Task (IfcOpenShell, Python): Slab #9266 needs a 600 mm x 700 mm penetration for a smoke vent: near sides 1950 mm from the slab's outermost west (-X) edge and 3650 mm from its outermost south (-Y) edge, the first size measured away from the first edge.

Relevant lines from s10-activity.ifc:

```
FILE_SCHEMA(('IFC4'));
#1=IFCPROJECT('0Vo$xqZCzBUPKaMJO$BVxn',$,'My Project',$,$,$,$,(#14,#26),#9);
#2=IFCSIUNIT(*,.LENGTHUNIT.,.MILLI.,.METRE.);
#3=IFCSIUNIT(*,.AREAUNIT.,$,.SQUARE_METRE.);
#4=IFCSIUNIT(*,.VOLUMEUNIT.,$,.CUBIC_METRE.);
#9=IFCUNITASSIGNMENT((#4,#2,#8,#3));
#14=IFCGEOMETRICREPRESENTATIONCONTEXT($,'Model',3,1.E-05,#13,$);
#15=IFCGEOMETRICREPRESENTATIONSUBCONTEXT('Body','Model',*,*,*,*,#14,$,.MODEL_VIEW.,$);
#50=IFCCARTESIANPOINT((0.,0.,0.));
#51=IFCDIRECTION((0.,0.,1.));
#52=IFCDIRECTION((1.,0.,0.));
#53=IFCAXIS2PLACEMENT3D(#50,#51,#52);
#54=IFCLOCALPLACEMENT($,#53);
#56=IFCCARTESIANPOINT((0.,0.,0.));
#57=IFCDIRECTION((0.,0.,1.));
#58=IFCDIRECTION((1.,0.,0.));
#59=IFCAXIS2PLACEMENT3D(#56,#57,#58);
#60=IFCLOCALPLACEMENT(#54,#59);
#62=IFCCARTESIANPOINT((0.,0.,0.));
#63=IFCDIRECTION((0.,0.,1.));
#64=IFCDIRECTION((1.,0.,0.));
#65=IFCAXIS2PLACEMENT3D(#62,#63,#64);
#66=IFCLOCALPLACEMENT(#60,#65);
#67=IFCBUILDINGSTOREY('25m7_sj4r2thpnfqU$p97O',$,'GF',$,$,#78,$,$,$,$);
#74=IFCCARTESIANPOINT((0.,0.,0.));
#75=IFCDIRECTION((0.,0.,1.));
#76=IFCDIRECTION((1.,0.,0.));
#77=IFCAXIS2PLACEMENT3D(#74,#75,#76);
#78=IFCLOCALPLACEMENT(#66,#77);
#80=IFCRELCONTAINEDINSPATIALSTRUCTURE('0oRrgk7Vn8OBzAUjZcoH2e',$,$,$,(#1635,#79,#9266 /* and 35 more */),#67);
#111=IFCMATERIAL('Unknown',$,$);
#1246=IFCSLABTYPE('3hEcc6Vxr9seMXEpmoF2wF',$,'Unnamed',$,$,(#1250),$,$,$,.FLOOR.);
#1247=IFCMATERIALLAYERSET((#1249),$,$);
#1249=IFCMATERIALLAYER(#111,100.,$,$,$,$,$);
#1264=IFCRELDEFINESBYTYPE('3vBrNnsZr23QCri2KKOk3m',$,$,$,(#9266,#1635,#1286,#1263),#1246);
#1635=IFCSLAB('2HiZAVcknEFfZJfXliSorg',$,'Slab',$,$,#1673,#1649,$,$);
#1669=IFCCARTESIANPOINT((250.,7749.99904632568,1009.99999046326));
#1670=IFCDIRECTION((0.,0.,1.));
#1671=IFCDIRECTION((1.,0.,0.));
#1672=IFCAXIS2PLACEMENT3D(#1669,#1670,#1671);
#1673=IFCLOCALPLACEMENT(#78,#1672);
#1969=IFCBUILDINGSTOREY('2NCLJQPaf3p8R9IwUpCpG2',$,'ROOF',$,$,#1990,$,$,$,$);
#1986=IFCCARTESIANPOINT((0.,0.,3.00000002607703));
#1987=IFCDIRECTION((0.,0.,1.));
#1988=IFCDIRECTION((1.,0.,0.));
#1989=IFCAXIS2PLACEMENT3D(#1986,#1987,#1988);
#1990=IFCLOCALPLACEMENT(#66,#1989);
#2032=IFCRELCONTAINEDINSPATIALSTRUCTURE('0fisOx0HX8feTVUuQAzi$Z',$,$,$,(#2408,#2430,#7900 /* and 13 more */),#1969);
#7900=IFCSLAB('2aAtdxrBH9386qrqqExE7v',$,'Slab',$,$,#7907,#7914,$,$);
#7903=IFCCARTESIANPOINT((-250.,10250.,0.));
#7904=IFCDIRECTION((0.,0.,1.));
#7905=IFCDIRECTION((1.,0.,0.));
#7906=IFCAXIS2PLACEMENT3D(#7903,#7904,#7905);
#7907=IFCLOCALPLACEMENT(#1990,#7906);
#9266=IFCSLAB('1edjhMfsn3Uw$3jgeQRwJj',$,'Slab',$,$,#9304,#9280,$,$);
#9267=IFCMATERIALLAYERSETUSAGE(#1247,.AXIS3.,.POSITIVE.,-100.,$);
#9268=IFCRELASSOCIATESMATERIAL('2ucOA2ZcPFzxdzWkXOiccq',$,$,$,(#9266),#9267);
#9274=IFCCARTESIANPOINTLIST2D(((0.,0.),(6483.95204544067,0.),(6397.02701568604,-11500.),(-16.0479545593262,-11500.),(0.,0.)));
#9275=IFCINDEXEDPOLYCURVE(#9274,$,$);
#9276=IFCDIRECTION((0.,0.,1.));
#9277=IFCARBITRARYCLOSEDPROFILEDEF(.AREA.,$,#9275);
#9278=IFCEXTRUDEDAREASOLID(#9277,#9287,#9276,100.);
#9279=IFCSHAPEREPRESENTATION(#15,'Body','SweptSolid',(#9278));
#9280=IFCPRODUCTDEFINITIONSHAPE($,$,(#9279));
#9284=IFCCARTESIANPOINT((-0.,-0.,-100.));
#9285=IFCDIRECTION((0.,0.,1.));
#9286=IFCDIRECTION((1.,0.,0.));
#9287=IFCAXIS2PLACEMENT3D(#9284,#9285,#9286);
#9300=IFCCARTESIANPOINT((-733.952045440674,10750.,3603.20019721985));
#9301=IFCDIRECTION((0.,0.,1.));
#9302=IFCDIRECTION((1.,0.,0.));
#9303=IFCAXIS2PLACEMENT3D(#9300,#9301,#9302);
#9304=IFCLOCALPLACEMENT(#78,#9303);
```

```python
import numpy as np
import ifcopenshell
import ifcopenshell.api.feature
import ifcopenshell.api.geometry
import ifcopenshell.api.root
import ifcopenshell.geom
import ifcopenshell.util.placement
import ifcopenshell.util.representation
import ifcopenshell.util.shape
import ifcopenshell.util.unit

model = ifcopenshell.open("s10-activity.ifc")
unit_scale = ifcopenshell.util.unit.calculate_unit_scale(model)
settings = ifcopenshell.geom.settings()


def volume(element):
    """Net volume in cubic metres, openings subtracted."""
    shape = ifcopenshell.geom.create_shape(settings, element)
    return ifcopenshell.util.shape.get_volume(shape.geometry)


slab = model.by_id(9266)
before = volume(slab)

# Extent in the slab's own axes, in metres. The edges named are its -X and -Y sides.
slab_shape = ifcopenshell.geom.create_shape(settings, slab)
vertices = ifcopenshell.util.shape.get_vertices(slab_shape.geometry)
x_min, y_min, bottom = vertices.min(axis=0)
top = vertices[:, 2].max()

opening = ifcopenshell.api.root.create_entity(model, ifc_class="IfcOpeningElement", name="Smoke vent opening", predefined_type="OPENING")
context = ifcopenshell.util.representation.get_context(model, "Model", "Body", "MODEL_VIEW")
width, depth = 0.6, 0.7
outline = [(0.0, 0.0), (width, 0.0), (width, depth), (0.0, depth), (0.0, 0.0)]
# Overshoot both faces by 50 mm so the cut is clean.
shape = ifcopenshell.api.geometry.add_slab_representation(
    model, context=context, depth=top - bottom + 0.1, polyline=outline
)
ifcopenshell.api.geometry.assign_representation(model, product=opening, representation=shape)

matrix = ifcopenshell.util.placement.get_local_placement(slab.ObjectPlacement)
matrix[:, 3] = matrix @ np.append(np.array([x_min + 1.95, y_min + 3.65, bottom - 0.05]) / unit_scale, 1.0)
ifcopenshell.api.geometry.edit_object_placement(model, product=opening, matrix=matrix, is_si=False)
ifcopenshell.api.feature.add_feature(model, feature=opening, element=slab)

after = volume(slab)

print(f"slab volume {before:.3f} -> {after:.3f} m3")

model.write("s10-activity_edited.ifc")
```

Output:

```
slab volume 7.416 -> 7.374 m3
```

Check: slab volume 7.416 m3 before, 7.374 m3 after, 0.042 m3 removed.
